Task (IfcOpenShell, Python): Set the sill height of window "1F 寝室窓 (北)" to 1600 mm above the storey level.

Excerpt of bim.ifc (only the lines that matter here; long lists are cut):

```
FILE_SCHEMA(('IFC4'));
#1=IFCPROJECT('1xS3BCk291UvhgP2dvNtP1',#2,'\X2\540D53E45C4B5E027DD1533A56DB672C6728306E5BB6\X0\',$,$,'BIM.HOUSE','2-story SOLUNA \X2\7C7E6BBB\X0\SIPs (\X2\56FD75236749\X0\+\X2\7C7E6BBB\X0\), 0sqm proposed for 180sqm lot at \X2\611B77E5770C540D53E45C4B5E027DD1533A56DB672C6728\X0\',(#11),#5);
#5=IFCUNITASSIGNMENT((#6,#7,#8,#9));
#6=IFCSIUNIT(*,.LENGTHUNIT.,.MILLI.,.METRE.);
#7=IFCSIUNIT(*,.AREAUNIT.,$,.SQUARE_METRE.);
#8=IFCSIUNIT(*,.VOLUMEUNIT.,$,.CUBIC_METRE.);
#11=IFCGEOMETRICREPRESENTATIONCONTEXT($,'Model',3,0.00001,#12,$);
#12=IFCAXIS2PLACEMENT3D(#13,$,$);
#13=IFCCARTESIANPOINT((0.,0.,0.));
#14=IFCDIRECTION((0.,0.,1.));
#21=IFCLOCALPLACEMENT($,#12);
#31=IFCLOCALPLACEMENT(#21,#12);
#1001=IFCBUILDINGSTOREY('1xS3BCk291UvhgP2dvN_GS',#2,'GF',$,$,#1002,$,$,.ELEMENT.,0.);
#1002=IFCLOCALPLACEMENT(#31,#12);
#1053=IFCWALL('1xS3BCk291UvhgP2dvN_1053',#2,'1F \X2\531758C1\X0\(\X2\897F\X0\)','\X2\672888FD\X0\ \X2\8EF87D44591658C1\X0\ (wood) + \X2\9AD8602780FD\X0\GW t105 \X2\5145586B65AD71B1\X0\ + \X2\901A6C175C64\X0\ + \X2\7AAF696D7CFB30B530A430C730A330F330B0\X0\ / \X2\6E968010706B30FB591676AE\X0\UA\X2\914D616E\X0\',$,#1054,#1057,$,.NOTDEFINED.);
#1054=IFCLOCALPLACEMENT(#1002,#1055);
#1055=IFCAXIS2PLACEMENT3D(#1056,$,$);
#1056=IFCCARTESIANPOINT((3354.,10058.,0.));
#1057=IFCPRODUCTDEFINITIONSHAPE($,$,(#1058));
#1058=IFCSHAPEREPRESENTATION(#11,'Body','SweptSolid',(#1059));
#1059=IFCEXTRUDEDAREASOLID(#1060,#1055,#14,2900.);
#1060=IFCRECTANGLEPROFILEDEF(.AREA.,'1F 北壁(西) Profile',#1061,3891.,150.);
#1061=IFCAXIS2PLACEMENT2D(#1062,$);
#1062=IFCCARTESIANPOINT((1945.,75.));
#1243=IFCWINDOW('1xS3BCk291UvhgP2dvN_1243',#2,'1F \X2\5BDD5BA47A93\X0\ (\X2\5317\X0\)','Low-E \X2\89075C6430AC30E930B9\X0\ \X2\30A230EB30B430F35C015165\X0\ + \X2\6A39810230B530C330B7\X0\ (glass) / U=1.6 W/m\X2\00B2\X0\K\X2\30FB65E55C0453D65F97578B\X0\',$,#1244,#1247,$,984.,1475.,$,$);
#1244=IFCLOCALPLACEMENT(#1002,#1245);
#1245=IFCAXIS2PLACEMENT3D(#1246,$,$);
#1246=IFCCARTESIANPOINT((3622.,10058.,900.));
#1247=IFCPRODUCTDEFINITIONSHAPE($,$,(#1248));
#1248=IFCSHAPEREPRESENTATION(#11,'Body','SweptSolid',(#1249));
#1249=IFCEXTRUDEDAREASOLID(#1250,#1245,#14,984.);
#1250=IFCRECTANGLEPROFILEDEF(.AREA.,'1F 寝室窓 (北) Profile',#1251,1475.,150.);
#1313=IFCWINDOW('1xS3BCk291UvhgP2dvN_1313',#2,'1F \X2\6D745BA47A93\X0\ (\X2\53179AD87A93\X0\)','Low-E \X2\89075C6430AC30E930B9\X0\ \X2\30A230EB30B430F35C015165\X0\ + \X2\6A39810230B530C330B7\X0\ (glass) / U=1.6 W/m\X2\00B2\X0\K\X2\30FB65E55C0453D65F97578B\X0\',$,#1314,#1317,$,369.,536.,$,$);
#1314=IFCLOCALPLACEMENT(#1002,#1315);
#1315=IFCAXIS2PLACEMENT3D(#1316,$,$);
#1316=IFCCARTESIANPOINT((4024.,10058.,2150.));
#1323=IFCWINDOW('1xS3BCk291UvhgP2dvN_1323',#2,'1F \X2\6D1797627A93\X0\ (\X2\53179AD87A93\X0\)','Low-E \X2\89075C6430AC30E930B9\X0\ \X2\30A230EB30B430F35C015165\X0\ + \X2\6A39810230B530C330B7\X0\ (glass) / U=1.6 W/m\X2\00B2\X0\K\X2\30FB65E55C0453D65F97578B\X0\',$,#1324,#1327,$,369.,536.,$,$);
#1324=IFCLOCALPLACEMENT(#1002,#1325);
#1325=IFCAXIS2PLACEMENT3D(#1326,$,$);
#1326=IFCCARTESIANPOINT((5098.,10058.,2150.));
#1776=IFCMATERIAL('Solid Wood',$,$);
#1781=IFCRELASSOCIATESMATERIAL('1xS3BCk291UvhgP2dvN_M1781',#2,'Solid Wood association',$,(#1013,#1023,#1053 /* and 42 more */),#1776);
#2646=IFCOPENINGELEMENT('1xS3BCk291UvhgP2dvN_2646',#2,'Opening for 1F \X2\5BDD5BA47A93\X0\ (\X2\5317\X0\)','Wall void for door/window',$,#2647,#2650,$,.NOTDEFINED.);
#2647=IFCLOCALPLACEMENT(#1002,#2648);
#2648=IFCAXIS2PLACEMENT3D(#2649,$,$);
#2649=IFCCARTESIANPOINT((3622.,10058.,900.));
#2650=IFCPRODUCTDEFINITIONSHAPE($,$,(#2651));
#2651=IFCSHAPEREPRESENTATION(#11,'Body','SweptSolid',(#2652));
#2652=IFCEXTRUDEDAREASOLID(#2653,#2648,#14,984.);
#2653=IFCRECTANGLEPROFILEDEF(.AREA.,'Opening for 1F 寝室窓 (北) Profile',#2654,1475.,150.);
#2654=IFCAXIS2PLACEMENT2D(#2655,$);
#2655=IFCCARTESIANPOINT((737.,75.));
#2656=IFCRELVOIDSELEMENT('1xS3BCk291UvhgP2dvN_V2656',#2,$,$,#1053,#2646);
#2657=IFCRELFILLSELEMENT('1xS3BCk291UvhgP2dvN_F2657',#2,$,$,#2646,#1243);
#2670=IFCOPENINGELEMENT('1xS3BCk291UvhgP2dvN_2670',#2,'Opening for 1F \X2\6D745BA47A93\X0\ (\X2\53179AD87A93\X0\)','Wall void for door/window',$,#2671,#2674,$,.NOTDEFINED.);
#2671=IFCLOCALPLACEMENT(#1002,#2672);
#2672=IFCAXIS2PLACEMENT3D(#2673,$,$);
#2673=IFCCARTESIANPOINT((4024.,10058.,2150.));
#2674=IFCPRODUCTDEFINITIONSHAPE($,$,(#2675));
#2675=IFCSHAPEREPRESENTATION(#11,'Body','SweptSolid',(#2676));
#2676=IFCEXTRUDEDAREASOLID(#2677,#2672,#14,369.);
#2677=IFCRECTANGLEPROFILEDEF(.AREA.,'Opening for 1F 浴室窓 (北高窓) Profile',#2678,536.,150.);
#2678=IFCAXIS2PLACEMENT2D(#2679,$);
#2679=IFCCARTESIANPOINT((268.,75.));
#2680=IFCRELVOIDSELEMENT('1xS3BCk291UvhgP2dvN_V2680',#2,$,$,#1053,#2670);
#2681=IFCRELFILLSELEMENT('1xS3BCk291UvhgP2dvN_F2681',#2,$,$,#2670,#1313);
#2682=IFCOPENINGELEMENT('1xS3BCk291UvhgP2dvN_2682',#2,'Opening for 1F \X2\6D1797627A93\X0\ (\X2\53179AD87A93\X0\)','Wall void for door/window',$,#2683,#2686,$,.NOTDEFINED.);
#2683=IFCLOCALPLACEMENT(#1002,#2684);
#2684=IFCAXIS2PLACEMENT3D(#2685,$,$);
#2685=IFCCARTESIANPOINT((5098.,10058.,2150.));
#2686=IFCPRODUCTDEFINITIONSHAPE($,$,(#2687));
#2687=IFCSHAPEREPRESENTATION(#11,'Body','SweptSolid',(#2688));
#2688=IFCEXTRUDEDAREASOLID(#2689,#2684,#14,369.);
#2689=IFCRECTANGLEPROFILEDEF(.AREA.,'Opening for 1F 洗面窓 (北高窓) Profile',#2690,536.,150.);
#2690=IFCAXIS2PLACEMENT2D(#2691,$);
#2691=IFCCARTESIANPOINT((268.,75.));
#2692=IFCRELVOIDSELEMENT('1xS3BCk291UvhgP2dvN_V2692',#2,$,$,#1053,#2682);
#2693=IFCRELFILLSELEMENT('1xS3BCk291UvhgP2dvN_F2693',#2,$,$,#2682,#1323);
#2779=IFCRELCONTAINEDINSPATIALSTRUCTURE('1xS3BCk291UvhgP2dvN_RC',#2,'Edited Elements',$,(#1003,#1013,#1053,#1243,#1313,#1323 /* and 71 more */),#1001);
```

```python
import numpy as np
import ifcopenshell
import ifcopenshell.api.geometry
import ifcopenshell.geom
import ifcopenshell.util.element
import ifcopenshell.util.placement
import ifcopenshell.util.shape
import ifcopenshell.util.unit

model = ifcopenshell.open("bim.ifc")
unit_scale = ifcopenshell.util.unit.calculate_unit_scale(model)

window = model.by_id(1243)
opening = window.FillsVoids[0].RelatingOpeningElement
storey = ifcopenshell.util.element.get_container(window, ifc_class="IfcBuildingStorey")
level = ifcopenshell.util.placement.get_local_placement(storey.ObjectPlacement)[2, 3]

# The opening's origin need not be at the sill, so measure its lowest point.
shape = ifcopenshell.geom.create_shape(ifcopenshell.geom.settings(), opening)
bottom = ifcopenshell.util.shape.get_shape_bottom_elevation(shape, shape.geometry) / unit_scale
dz = level + 1.6 / unit_scale - bottom

shift = np.array([0.0, 0.0, dz])
# The window is not placed relative to its opening, so move both.
for product in (opening, window):
    matrix = ifcopenshell.util.placement.get_local_placement(product.ObjectPlacement)
    matrix[:3, 3] += shift
    ifcopenshell.api.geometry.edit_object_placement(model, product=product, matrix=matrix, is_si=False)

print(f"moved by {dz * unit_scale:+.3f} m")

model.write("bim_updated.ifc")
```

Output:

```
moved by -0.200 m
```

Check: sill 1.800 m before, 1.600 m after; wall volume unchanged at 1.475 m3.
